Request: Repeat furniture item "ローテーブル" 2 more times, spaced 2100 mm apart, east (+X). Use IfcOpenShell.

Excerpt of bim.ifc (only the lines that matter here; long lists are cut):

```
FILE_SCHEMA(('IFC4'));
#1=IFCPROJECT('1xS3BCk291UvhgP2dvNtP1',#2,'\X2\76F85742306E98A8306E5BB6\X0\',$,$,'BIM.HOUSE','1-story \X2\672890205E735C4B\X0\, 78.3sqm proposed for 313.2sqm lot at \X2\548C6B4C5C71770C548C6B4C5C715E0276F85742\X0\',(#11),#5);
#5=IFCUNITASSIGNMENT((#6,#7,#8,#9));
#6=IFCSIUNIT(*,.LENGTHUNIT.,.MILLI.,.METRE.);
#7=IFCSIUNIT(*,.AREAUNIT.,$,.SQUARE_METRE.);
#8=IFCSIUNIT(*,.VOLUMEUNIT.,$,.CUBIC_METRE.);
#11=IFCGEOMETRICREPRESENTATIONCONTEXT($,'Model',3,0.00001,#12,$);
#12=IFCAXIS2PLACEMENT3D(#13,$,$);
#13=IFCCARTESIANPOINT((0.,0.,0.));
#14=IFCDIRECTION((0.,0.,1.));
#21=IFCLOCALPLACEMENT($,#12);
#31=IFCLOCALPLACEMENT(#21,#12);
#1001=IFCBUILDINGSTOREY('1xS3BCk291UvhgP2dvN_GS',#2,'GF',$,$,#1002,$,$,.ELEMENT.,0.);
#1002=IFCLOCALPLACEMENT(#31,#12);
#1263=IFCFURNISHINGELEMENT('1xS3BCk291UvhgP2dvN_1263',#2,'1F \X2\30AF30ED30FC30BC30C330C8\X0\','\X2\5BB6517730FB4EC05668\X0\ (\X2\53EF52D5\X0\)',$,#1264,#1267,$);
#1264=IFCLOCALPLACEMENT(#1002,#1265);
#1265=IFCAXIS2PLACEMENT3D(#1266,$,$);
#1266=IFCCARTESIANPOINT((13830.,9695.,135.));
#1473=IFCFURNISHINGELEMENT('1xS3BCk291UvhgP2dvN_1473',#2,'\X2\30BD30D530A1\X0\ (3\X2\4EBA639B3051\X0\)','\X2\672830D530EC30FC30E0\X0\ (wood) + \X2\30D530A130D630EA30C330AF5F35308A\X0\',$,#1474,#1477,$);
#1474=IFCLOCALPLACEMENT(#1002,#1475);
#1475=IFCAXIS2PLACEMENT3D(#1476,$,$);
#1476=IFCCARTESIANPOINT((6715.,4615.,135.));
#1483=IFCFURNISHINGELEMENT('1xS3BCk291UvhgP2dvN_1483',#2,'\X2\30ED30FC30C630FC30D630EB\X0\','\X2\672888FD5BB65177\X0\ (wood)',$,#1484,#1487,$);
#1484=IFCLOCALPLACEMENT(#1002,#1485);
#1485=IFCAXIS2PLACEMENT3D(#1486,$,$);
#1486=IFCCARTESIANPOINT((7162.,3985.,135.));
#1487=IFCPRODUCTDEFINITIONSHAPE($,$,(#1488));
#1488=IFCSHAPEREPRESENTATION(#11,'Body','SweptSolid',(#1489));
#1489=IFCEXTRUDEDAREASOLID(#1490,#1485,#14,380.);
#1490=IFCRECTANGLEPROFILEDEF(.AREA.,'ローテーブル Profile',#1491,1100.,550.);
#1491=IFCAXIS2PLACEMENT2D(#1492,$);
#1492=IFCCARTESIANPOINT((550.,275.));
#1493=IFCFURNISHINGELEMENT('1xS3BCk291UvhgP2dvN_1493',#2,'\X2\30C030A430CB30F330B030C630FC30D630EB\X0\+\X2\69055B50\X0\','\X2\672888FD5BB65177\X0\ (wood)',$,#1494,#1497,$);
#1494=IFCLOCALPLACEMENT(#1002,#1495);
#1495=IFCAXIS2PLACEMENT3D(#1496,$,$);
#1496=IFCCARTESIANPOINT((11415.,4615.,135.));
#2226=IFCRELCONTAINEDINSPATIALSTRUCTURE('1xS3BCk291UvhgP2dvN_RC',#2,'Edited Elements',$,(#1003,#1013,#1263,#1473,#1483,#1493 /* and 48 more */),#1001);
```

```python
import numpy as np
import ifcopenshell
import ifcopenshell.api.geometry
import ifcopenshell.api.root
import ifcopenshell.util.element
import ifcopenshell.util.placement

model = ifcopenshell.open("bim.ifc")


def reuse_history(source, copy):
    """copy_class also copies each property set's owner history, people and application; keep the originals."""
    for rel in copy.IsDefinedBy:
        if rel.is_a("IfcRelDefinesByProperties") and (history := rel.RelatingPropertyDefinition.OwnerHistory):
            rel.RelatingPropertyDefinition.OwnerHistory = source.OwnerHistory
            ifcopenshell.util.element.remove_deep2(model, history)


source = model.by_guid("1xS3BCk291UvhgP2dvN_1483")
base = ifcopenshell.util.placement.get_local_placement(source.ObjectPlacement)
step = np.array([1.0, 0.0, 0.0]) * 2100.0

for i in range(1, 3):
    copy = ifcopenshell.api.root.copy_class(model, product=source)
    copy.Representation = ifcopenshell.util.element.copy_deep(
        model, source.Representation, exclude=["IfcGeometricRepresentationContext", "IfcRepresentationMap"]
    )
    reuse_history(source, copy)
    matrix = base.copy()
    matrix[:3, 3] += i * step
    print("added at", matrix[:3, 3].round(3) + 0.0)
    ifcopenshell.api.geometry.edit_object_placement(model, product=copy, matrix=matrix, is_si=False)

model.write("bim_updated.ifc")
```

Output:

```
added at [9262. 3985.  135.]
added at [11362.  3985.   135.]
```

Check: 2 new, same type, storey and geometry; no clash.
